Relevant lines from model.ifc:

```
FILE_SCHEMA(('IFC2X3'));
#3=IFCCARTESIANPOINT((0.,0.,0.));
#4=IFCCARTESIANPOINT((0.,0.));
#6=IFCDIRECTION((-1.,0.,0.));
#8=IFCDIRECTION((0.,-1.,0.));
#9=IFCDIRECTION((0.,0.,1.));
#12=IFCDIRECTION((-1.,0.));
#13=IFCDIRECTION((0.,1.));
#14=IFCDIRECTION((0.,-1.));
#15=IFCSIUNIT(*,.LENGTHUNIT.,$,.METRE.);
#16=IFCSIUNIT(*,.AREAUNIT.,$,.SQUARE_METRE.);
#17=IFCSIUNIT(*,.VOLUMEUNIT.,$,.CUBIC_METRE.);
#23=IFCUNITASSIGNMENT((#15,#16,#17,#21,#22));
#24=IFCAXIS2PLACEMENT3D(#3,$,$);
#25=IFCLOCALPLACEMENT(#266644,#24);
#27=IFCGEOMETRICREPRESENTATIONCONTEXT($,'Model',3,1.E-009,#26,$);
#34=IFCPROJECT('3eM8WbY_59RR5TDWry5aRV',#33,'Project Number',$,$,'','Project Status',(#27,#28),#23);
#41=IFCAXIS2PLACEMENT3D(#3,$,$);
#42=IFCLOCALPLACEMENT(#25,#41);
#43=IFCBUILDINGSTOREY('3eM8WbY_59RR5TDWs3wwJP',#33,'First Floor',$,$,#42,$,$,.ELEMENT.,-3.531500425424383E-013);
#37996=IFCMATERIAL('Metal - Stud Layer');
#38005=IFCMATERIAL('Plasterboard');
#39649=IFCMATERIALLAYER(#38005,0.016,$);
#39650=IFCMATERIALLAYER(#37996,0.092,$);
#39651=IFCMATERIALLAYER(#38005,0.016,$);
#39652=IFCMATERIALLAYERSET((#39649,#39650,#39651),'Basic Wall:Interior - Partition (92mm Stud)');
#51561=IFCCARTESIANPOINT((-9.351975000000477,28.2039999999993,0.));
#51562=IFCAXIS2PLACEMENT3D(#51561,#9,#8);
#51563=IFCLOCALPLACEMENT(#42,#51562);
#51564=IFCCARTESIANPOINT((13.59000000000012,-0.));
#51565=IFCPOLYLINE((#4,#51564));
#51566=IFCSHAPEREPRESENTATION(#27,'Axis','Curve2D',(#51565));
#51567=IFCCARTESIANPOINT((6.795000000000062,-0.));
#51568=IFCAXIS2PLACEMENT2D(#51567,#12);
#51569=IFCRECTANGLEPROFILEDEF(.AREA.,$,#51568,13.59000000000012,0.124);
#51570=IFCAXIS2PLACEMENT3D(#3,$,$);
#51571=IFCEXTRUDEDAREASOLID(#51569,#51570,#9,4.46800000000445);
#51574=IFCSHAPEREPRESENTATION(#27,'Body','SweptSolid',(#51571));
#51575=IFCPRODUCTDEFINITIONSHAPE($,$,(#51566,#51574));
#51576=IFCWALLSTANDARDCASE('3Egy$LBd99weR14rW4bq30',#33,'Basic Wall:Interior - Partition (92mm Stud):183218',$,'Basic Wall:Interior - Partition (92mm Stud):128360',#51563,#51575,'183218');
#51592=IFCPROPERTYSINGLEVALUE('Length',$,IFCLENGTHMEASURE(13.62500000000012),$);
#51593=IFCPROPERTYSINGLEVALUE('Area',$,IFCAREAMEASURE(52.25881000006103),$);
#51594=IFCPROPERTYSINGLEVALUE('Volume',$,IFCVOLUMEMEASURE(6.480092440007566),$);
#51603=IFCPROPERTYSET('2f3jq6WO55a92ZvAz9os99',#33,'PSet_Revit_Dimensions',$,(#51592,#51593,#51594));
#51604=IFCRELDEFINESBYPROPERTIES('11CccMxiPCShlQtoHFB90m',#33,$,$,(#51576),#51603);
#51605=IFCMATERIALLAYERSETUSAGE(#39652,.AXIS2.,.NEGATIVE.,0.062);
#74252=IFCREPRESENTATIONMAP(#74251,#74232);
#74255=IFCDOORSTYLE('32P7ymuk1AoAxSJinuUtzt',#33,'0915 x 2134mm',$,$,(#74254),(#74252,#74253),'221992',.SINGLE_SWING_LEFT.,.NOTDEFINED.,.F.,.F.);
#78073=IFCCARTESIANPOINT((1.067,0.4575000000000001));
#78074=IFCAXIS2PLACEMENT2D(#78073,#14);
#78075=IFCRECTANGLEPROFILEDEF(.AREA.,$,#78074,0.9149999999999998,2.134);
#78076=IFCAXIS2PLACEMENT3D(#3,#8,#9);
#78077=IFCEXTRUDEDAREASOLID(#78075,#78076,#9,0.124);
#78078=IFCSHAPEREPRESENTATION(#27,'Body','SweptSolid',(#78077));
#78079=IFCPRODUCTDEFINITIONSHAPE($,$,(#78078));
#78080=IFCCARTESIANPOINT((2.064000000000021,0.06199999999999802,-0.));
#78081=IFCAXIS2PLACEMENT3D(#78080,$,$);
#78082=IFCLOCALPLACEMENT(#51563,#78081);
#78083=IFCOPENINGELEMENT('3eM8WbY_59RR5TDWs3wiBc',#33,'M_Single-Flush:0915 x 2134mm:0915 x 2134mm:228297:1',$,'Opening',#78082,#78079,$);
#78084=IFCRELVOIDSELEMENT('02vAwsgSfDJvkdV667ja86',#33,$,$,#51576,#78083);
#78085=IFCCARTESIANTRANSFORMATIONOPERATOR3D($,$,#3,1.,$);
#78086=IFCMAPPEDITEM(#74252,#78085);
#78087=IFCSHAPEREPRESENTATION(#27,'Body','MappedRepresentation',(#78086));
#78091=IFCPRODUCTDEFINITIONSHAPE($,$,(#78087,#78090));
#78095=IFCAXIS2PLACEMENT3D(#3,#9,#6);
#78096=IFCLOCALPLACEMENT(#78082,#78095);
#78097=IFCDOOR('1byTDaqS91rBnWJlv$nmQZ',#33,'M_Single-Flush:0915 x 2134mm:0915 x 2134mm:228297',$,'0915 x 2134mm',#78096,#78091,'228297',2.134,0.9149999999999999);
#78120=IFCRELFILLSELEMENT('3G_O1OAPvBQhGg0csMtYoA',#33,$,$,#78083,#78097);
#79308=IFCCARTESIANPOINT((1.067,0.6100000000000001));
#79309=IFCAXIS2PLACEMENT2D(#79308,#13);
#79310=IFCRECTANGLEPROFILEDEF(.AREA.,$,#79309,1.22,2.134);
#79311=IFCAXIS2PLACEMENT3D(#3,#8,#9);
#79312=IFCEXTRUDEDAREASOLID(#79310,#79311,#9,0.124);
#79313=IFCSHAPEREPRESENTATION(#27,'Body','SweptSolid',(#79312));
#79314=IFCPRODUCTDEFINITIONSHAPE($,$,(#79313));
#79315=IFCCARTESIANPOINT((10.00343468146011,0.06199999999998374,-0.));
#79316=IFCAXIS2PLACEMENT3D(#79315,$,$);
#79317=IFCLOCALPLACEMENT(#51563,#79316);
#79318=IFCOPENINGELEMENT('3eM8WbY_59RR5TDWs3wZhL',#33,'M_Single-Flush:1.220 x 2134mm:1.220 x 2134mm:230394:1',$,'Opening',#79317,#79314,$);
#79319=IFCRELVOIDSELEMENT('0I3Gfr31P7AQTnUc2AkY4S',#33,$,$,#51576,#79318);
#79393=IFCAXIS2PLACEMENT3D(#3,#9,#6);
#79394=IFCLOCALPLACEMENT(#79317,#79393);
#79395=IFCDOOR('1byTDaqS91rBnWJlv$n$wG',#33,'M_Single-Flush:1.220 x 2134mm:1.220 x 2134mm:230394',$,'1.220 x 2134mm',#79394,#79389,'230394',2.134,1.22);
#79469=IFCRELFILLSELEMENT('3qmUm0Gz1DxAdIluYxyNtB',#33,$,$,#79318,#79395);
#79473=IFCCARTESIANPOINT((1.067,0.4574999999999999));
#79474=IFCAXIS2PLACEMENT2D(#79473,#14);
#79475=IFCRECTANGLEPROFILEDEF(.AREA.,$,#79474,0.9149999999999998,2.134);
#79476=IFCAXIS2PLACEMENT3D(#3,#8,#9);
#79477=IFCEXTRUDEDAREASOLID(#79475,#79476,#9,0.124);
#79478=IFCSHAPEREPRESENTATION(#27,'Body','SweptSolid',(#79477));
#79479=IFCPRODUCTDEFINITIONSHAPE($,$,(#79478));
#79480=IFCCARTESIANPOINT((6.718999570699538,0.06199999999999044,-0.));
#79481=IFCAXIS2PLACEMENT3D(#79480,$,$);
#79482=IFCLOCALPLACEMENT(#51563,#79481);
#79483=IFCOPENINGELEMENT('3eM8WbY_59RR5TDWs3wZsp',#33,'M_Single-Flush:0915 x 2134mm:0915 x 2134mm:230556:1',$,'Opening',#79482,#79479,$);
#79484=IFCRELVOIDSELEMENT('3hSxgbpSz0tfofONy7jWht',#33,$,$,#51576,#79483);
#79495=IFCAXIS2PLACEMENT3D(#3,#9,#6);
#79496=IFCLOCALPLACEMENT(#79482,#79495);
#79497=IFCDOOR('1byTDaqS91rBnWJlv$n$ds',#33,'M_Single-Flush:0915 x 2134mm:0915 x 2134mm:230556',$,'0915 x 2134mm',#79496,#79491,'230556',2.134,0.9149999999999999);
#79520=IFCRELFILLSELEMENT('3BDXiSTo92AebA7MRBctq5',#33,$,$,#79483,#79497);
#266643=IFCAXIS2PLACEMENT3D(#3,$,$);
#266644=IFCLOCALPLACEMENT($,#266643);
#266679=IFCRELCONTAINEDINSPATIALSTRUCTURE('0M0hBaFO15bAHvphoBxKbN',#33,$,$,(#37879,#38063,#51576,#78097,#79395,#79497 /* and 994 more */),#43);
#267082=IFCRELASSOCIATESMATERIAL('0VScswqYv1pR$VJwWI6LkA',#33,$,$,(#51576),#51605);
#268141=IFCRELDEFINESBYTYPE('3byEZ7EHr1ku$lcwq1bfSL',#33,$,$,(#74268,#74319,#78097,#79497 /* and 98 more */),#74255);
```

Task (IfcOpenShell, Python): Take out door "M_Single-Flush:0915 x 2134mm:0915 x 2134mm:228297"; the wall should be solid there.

```python
import ifcopenshell
import ifcopenshell.api.feature
import ifcopenshell.api.pset
import ifcopenshell.api.root
import ifcopenshell.geom
import ifcopenshell.util.element
import ifcopenshell.util.shape
import ifcopenshell.util.unit

model = ifcopenshell.open("model.ifc")
area_scale = ifcopenshell.util.unit.calculate_unit_scale(model, "AREAUNIT")
volume_scale = ifcopenshell.util.unit.calculate_unit_scale(model, "VOLUMEUNIT")
settings = ifcopenshell.geom.settings()


def volume(element):
    """Net volume in cubic metres, openings subtracted."""
    shape = ifcopenshell.geom.create_shape(settings, element)
    return ifcopenshell.util.shape.get_volume(shape.geometry)


door = model.by_guid("1byTDaqS91rBnWJlv$nmQZ")
opening = door.FillsVoids[0].RelatingOpeningElement
wall = opening.VoidsElements[0].RelatingBuildingElement
before = volume(wall)

ifcopenshell.api.root.remove_product(model, product=door)
ifcopenshell.api.feature.remove_feature(model, feature=opening)

after = volume(wall)
thickness = 0.124  # wall thickness in metres

# Update the wall's stored quantities.
pset = model.by_id(ifcopenshell.util.element.get_pset(wall, "PSet_Revit_Dimensions", should_inherit=False)["id"])
ifcopenshell.api.pset.edit_pset(model, pset=pset, properties={
    "Area": model.create_entity("IfcAreaMeasure", after / thickness / area_scale),
    "Volume": model.create_entity("IfcVolumeMeasure", after / volume_scale),
})

print(f"wall volume {before:.3f} -> {after:.3f} m3")

model.write("model_rev.ifc")
```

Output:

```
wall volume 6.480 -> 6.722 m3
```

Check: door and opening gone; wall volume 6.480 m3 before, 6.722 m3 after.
